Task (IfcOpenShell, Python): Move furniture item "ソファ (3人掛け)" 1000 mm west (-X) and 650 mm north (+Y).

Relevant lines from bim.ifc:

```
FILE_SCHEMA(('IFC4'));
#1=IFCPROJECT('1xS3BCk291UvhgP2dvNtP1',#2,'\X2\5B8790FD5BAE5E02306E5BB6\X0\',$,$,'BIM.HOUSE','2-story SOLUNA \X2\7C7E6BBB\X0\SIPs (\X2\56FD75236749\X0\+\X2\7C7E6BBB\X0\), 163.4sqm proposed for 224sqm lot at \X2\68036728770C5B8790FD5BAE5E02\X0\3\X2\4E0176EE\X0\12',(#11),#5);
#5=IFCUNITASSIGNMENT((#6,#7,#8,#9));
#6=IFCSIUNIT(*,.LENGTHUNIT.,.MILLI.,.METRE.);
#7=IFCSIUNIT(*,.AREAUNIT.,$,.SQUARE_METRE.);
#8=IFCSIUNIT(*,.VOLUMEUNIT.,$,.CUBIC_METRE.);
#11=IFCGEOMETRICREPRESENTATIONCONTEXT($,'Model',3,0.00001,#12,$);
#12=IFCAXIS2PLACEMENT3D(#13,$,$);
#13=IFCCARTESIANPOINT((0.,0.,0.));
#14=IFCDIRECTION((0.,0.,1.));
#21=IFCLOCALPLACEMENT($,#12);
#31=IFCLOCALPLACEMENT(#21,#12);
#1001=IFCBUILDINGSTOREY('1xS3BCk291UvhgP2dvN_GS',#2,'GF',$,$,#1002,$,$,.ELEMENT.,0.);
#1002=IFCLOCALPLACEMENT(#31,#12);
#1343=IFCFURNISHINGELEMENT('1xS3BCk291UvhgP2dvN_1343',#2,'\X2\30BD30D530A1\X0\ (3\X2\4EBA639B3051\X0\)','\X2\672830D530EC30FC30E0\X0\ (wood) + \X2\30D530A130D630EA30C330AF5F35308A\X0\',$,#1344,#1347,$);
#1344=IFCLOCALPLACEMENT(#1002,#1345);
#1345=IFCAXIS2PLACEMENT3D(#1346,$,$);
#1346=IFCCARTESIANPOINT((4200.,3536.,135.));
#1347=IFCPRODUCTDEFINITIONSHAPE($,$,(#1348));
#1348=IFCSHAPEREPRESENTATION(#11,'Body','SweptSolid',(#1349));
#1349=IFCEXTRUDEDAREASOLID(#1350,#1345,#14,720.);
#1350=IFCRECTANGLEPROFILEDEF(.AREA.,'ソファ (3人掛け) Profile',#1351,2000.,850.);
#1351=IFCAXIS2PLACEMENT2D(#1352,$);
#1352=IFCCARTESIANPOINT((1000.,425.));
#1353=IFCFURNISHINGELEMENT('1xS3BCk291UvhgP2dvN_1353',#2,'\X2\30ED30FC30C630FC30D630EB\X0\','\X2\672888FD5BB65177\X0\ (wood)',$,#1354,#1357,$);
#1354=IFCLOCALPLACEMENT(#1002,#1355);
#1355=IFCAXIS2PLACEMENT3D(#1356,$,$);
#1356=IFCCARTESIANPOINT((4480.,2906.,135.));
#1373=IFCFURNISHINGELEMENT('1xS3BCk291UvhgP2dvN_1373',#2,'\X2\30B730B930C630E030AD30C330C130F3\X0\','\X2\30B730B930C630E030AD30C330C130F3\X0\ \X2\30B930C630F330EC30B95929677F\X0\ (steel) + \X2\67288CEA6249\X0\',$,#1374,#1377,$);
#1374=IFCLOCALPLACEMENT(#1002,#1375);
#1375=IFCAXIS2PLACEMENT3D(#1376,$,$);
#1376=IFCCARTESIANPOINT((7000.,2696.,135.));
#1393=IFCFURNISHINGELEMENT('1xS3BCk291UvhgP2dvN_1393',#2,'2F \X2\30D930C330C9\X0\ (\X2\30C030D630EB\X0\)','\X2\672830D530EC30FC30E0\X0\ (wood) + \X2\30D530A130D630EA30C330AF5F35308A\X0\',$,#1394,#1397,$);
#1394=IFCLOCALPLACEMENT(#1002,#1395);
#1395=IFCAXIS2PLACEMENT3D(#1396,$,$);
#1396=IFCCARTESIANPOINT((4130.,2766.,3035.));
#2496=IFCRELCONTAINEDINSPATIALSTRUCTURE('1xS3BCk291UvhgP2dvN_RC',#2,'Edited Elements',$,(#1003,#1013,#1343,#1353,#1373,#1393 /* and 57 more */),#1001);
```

```python
import ifcopenshell
import ifcopenshell.api.geometry
import ifcopenshell.util.placement
import ifcopenshell.util.unit

model = ifcopenshell.open("bim.ifc")
unit_scale = ifcopenshell.util.unit.calculate_unit_scale(model)

item = model.by_guid("1xS3BCk291UvhgP2dvN_1343")
matrix = ifcopenshell.util.placement.get_local_placement(item.ObjectPlacement)
matrix[0, 3] -= 1 / unit_scale
matrix[1, 3] += 0.65 / unit_scale
ifcopenshell.api.geometry.edit_object_placement(model, product=item, matrix=matrix, is_si=False)

print(ifcopenshell.util.placement.get_local_placement(item.ObjectPlacement).round(3) + 0.0)

model.write("bim_rev.ifc")
```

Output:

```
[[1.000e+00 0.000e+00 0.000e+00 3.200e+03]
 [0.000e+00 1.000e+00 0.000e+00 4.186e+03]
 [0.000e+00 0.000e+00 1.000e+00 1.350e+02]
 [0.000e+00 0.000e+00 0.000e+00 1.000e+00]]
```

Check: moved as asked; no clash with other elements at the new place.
